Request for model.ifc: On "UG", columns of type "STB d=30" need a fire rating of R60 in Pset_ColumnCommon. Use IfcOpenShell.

First a look at what the model holds.

```python
import ifcopenshell
import ifcopenshell.util.element

model = ifcopenshell.open("model.ifc")
print(model.schema)
storey = next(s for s in model.by_type("IfcBuildingStorey") if s.Name == "UG")
columns = [e for e in ifcopenshell.util.element.get_decomposition(storey) if e.is_a("IfcColumn")]
seen = {}
for e in columns:
    element_type = ifcopenshell.util.element.get_type(e)
    key = (element_type.Name if element_type != e and element_type else None, ifcopenshell.util.element.get_pset(e, "Pset_ColumnCommon", "FireRating"))
    seen[key] = seen.get(key, 0) + 1
for (name, value), count in sorted(seen.items(), key=str):
    print(count, "x", name, "|", value)
```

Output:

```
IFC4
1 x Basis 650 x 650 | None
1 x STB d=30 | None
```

```python
import ifcopenshell
import ifcopenshell.api.pset
import ifcopenshell.util.element

model = ifcopenshell.open("model.ifc")

storey = next(s for s in model.by_type("IfcBuildingStorey") if s.Name == "UG")
columns = [e for e in ifcopenshell.util.element.get_decomposition(storey) if e.is_a("IfcColumn")]

count = 0
for e in columns:
    element_type = ifcopenshell.util.element.get_type(e)
    if element_type in (None, e) or element_type.Name != "STB d=30":
        continue
    # add_pset returns the element's existing set when there is one.
    pset = ifcopenshell.api.pset.add_pset(model, product=e, name="Pset_ColumnCommon")
    ifcopenshell.api.pset.edit_pset(model, pset=pset, properties={"FireRating": "R60"})
    count += 1

print(count, "columns updated")

model.write("model_rev.ifc")
```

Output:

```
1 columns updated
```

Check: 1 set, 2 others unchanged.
